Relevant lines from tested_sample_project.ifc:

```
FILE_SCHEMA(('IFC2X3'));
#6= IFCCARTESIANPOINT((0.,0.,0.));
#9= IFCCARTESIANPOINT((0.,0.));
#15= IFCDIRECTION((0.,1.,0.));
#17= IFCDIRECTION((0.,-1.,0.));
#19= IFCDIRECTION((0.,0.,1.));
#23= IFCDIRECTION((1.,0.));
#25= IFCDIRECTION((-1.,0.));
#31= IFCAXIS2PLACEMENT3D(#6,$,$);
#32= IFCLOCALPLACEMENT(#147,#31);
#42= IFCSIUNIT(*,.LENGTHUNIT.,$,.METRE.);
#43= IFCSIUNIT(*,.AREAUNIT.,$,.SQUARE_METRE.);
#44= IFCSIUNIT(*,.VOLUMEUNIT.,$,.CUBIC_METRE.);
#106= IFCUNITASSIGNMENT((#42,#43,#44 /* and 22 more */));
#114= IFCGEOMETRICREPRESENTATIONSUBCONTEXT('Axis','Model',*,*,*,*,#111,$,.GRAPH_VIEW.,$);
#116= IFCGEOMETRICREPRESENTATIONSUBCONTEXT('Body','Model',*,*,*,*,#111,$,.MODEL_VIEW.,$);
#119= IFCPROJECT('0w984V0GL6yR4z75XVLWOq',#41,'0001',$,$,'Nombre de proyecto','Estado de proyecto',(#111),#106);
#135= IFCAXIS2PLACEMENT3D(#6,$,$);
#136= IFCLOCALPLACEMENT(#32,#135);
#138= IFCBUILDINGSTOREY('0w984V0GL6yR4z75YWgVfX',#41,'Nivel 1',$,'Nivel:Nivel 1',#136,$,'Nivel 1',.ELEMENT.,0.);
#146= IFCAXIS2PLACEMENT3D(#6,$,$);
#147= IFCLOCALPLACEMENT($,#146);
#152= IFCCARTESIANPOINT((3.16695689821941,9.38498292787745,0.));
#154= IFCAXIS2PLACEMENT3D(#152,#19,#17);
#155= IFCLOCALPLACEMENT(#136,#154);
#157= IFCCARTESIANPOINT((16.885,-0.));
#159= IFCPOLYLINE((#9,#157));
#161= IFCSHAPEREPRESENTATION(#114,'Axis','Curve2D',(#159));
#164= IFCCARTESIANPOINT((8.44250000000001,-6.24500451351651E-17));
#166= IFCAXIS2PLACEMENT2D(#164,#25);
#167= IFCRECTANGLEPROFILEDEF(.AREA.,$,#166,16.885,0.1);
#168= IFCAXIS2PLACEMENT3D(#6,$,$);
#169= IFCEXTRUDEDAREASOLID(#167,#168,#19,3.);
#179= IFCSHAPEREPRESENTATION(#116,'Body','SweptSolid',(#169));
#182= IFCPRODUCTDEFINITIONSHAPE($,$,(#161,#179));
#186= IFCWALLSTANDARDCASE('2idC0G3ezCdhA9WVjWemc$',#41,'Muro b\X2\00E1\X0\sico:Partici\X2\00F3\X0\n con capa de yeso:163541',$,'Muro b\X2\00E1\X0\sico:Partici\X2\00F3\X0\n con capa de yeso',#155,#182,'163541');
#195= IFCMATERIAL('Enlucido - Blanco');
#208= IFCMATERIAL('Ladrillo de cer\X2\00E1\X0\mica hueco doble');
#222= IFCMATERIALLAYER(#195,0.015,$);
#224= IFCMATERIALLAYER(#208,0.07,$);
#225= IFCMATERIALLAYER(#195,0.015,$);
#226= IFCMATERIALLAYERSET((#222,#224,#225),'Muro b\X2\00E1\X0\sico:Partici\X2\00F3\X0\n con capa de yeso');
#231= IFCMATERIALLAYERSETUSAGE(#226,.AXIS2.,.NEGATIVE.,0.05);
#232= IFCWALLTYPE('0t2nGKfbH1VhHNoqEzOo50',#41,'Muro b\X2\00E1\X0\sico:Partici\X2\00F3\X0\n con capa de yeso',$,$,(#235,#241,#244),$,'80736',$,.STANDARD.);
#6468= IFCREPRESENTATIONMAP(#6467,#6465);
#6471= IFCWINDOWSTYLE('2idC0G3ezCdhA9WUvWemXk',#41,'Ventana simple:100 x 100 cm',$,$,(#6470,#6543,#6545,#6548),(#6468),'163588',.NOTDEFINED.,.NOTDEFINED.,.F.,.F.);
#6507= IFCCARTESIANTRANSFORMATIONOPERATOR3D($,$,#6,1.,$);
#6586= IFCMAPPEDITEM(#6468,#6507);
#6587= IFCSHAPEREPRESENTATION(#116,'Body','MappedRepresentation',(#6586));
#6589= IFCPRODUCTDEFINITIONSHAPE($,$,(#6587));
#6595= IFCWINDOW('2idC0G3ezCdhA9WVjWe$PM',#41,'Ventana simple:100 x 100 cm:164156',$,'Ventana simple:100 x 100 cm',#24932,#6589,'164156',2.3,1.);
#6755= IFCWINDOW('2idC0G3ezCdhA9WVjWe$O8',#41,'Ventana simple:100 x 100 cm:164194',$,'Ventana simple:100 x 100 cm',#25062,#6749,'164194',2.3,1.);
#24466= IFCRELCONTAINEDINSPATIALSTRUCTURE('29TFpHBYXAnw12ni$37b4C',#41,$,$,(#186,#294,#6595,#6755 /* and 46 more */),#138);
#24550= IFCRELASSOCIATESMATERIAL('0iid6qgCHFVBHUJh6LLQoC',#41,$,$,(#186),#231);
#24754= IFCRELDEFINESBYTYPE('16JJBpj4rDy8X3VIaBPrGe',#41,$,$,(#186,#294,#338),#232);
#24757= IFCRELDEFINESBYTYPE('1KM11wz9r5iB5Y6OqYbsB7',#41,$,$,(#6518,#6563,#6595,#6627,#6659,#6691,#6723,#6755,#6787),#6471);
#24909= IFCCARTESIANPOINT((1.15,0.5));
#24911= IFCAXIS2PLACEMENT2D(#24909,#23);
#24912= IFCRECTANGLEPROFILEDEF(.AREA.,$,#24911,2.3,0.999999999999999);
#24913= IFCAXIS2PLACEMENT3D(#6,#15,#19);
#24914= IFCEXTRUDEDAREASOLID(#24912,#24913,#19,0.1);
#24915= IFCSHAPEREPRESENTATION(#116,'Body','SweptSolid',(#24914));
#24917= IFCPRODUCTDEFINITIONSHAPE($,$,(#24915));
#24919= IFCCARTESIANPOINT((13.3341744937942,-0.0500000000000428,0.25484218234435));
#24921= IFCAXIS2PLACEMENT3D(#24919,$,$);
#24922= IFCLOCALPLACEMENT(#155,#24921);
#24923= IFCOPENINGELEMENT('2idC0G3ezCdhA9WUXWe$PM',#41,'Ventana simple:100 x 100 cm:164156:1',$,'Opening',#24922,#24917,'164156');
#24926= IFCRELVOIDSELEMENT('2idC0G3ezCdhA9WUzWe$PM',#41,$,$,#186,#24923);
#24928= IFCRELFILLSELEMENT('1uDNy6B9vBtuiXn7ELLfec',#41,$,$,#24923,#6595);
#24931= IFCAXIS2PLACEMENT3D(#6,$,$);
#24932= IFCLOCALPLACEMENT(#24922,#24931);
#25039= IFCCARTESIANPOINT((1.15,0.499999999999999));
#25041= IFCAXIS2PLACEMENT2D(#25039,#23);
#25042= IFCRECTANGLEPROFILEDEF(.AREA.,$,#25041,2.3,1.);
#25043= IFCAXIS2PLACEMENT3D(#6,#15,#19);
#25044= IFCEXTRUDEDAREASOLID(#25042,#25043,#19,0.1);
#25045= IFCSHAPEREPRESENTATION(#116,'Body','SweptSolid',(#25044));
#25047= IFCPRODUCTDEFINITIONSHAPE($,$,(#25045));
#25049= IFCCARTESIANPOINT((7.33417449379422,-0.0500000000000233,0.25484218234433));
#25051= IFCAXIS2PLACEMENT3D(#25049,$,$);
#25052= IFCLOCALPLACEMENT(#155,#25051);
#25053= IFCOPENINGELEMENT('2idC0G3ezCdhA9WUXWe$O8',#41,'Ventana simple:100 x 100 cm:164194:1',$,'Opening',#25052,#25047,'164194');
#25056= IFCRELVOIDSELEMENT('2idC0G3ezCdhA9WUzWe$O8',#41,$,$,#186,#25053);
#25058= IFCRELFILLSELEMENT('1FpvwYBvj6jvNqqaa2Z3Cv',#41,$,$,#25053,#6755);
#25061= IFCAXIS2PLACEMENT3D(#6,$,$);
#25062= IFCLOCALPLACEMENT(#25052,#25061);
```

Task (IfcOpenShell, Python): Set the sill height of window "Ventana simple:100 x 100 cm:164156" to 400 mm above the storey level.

```python
import numpy as np
import ifcopenshell
import ifcopenshell.api.geometry
import ifcopenshell.geom
import ifcopenshell.util.element
import ifcopenshell.util.placement
import ifcopenshell.util.shape
import ifcopenshell.util.unit

model = ifcopenshell.open("tested_sample_project.ifc")
unit_scale = ifcopenshell.util.unit.calculate_unit_scale(model)

window = model.by_id(6595)
opening = window.FillsVoids[0].RelatingOpeningElement
storey = ifcopenshell.util.element.get_container(window, ifc_class="IfcBuildingStorey")
level = ifcopenshell.util.placement.get_local_placement(storey.ObjectPlacement)[2, 3]

# The opening's origin need not be at the sill, so measure its lowest point.
shape = ifcopenshell.geom.create_shape(ifcopenshell.geom.settings(), opening)
bottom = ifcopenshell.util.shape.get_shape_bottom_elevation(shape, shape.geometry) / unit_scale
dz = level + 0.4 / unit_scale - bottom

shift = np.array([0.0, 0.0, dz])
# The window is placed relative to its opening, so it follows when the opening moves.
matrix = ifcopenshell.util.placement.get_local_placement(opening.ObjectPlacement)
matrix[:3, 3] += shift
ifcopenshell.api.geometry.edit_object_placement(
    model, product=opening, matrix=matrix, is_si=False, should_transform_children=True
)

print(f"moved by {dz * unit_scale:+.3f} m")

model.write("tested_sample_project_updated.ifc")
```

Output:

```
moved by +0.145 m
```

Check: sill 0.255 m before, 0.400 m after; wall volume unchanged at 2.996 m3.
